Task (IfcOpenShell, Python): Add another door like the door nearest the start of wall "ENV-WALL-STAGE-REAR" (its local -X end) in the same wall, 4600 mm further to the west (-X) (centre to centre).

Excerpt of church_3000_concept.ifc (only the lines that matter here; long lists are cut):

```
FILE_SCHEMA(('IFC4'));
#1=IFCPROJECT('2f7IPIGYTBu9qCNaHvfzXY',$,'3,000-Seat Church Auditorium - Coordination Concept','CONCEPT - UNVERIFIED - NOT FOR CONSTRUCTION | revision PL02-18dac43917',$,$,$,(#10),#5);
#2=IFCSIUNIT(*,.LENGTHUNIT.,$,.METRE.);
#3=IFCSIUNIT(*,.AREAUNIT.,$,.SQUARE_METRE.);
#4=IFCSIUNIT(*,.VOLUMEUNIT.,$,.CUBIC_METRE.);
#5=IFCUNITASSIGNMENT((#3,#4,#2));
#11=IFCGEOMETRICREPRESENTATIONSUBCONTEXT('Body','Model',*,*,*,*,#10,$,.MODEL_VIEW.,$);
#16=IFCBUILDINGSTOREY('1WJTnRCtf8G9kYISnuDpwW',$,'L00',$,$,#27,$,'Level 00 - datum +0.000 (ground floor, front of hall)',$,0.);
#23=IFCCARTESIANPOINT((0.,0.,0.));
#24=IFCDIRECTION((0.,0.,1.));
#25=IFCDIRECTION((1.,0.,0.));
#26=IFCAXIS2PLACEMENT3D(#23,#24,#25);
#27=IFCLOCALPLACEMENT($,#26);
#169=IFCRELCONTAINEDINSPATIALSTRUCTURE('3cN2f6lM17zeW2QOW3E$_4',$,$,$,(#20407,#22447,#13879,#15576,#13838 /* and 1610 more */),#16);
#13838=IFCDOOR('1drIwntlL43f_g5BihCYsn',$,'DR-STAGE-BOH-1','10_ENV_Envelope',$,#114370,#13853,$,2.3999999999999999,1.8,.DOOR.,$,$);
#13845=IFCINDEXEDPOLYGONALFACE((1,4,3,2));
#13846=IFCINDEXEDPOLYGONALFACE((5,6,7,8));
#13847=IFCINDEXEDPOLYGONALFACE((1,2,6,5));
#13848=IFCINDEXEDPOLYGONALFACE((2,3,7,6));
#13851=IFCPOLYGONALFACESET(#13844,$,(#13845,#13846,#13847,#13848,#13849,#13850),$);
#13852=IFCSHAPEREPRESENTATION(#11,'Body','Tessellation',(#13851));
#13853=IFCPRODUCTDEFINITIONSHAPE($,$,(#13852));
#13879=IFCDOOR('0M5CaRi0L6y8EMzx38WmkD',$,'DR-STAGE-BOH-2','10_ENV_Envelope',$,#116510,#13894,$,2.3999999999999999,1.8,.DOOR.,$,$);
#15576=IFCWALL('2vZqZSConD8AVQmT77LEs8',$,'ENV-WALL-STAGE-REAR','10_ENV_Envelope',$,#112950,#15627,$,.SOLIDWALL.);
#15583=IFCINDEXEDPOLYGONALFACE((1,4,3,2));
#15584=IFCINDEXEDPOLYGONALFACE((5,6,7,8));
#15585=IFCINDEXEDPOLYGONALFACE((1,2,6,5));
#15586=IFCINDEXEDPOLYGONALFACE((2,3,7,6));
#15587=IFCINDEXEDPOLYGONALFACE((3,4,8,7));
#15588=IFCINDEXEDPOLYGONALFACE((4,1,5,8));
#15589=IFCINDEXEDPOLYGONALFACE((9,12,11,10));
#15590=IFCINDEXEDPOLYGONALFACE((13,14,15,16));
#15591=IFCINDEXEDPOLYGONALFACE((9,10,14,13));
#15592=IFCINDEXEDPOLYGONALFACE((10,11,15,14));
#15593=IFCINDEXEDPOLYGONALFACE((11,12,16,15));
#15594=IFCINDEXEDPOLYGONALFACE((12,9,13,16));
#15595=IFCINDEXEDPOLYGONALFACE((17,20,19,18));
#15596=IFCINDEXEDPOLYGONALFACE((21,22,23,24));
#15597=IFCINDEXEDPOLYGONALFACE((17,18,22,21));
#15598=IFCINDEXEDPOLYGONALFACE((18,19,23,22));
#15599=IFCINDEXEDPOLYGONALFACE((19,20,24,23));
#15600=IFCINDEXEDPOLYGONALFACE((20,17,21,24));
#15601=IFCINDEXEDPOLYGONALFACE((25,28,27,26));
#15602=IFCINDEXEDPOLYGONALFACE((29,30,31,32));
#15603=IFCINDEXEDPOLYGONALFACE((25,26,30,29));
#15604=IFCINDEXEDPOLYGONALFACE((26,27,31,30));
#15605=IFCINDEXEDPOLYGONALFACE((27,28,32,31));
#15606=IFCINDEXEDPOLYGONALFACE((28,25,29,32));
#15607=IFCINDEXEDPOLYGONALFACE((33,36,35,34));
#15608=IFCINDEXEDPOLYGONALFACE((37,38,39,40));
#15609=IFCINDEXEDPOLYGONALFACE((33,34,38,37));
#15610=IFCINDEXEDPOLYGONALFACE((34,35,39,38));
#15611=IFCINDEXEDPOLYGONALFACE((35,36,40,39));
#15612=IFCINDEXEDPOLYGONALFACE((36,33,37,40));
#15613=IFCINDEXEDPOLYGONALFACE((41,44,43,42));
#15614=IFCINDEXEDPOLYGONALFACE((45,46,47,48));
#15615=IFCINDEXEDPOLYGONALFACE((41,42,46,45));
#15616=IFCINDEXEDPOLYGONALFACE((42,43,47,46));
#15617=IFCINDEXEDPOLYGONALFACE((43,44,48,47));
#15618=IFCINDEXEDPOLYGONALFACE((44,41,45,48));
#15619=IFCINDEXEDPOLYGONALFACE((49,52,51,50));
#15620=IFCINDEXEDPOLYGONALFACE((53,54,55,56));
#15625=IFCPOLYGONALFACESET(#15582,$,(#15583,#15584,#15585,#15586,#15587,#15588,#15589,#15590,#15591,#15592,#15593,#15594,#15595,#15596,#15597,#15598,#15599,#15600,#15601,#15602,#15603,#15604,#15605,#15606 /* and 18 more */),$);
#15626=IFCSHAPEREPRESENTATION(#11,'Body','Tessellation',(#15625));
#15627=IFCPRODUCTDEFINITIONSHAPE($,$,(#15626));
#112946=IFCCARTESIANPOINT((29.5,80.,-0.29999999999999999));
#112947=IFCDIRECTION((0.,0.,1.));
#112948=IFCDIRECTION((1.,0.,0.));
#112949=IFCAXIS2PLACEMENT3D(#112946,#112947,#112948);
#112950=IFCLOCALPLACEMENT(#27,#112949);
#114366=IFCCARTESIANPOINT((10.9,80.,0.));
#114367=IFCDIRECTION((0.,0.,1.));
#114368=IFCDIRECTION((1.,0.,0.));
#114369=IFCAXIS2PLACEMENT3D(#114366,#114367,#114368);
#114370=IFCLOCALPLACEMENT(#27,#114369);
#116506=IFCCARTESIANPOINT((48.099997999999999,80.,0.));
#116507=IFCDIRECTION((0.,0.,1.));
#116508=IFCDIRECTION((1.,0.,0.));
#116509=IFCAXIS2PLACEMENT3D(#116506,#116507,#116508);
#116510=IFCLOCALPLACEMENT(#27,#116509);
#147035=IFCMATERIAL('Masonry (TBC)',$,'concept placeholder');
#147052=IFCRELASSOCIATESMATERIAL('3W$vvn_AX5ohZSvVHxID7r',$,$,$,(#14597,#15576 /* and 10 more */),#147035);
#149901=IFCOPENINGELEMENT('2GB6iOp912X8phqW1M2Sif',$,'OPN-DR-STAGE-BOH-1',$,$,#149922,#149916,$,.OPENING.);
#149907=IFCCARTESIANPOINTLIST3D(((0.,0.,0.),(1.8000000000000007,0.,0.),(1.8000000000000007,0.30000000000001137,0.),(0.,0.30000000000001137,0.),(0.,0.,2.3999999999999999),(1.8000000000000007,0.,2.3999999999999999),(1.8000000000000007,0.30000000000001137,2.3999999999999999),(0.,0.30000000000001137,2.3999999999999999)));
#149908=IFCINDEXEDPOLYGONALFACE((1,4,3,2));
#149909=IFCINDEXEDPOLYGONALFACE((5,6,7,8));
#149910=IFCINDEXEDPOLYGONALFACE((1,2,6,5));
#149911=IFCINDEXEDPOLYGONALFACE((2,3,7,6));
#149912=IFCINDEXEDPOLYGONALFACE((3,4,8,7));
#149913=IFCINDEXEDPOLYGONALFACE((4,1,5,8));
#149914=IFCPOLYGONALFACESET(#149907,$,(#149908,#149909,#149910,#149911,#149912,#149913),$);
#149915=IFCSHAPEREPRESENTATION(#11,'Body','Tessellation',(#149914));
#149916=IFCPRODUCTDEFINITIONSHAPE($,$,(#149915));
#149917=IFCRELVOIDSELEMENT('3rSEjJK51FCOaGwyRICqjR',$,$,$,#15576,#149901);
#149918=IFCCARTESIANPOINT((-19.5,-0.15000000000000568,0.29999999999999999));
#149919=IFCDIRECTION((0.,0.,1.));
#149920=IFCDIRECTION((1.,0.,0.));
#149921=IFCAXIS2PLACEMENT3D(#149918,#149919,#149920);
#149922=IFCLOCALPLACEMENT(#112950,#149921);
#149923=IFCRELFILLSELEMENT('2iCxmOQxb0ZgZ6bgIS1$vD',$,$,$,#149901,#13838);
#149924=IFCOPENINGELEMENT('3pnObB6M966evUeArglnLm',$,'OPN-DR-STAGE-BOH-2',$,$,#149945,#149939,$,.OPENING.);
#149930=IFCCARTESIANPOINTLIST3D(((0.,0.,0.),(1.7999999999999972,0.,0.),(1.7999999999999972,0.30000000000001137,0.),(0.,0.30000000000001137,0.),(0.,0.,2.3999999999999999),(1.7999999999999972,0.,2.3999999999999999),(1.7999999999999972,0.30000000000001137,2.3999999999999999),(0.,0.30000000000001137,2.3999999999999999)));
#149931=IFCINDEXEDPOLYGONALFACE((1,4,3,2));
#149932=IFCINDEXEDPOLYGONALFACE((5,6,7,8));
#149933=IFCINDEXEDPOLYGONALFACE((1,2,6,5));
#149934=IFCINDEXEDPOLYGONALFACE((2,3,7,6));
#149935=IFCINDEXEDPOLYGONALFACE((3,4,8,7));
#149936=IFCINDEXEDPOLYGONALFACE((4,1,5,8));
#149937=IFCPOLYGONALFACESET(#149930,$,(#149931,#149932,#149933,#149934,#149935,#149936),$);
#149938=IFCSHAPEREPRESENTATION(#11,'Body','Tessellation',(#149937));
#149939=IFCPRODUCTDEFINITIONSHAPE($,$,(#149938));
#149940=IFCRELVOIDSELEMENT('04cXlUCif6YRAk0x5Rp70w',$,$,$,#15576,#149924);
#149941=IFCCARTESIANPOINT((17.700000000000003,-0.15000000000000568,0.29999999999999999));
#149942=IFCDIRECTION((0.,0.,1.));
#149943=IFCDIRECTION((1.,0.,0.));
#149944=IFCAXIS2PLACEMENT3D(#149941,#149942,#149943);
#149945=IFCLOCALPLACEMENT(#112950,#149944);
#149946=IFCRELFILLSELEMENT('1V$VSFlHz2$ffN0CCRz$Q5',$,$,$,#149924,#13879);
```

```python
import ifcopenshell
import ifcopenshell.api.feature
import ifcopenshell.api.geometry
import ifcopenshell.api.root
import ifcopenshell.geom
import ifcopenshell.util.element
import ifcopenshell.util.placement
import ifcopenshell.util.shape

model = ifcopenshell.open("church_3000_concept.ifc")
settings = ifcopenshell.geom.settings()


def volume(element):
    """Net volume in cubic metres, openings subtracted."""
    shape = ifcopenshell.geom.create_shape(settings, element)
    return ifcopenshell.util.shape.get_volume(shape.geometry)


door = model.by_guid("1drIwntlL43f_g5BihCYsn")
opening = door.FillsVoids[0].RelatingOpeningElement
wall = opening.VoidsElements[0].RelatingBuildingElement
before = volume(wall)
shift = ifcopenshell.util.placement.get_local_placement(wall.ObjectPlacement)[:3, 0] * -4.6

# copy_class copies the void relationship, type, container and properties, but no geometry.
new_opening = ifcopenshell.api.root.copy_class(model, product=opening)
new_opening.Representation = ifcopenshell.util.element.copy_deep(
    model, opening.Representation, exclude=["IfcGeometricRepresentationContext", "IfcRepresentationMap"]
)
new_door = ifcopenshell.api.root.copy_class(model, product=door)
new_door.Representation = ifcopenshell.util.element.copy_deep(
    model, door.Representation, exclude=["IfcGeometricRepresentationContext", "IfcRepresentationMap"]
)
ifcopenshell.api.feature.add_filling(model, opening=new_opening, element=new_door)

for old, new in ((opening, new_opening), (door, new_door)):
    matrix = ifcopenshell.util.placement.get_local_placement(old.ObjectPlacement)
    matrix[:3, 3] += shift
    ifcopenshell.api.geometry.edit_object_placement(model, product=new, matrix=matrix, is_si=False)

after = volume(wall)

print(f"wall volume {before:.3f} -> {after:.3f} m3")

model.write("church_3000_concept-out.ifc")
```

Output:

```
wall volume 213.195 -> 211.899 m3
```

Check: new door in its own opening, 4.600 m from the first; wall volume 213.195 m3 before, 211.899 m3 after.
